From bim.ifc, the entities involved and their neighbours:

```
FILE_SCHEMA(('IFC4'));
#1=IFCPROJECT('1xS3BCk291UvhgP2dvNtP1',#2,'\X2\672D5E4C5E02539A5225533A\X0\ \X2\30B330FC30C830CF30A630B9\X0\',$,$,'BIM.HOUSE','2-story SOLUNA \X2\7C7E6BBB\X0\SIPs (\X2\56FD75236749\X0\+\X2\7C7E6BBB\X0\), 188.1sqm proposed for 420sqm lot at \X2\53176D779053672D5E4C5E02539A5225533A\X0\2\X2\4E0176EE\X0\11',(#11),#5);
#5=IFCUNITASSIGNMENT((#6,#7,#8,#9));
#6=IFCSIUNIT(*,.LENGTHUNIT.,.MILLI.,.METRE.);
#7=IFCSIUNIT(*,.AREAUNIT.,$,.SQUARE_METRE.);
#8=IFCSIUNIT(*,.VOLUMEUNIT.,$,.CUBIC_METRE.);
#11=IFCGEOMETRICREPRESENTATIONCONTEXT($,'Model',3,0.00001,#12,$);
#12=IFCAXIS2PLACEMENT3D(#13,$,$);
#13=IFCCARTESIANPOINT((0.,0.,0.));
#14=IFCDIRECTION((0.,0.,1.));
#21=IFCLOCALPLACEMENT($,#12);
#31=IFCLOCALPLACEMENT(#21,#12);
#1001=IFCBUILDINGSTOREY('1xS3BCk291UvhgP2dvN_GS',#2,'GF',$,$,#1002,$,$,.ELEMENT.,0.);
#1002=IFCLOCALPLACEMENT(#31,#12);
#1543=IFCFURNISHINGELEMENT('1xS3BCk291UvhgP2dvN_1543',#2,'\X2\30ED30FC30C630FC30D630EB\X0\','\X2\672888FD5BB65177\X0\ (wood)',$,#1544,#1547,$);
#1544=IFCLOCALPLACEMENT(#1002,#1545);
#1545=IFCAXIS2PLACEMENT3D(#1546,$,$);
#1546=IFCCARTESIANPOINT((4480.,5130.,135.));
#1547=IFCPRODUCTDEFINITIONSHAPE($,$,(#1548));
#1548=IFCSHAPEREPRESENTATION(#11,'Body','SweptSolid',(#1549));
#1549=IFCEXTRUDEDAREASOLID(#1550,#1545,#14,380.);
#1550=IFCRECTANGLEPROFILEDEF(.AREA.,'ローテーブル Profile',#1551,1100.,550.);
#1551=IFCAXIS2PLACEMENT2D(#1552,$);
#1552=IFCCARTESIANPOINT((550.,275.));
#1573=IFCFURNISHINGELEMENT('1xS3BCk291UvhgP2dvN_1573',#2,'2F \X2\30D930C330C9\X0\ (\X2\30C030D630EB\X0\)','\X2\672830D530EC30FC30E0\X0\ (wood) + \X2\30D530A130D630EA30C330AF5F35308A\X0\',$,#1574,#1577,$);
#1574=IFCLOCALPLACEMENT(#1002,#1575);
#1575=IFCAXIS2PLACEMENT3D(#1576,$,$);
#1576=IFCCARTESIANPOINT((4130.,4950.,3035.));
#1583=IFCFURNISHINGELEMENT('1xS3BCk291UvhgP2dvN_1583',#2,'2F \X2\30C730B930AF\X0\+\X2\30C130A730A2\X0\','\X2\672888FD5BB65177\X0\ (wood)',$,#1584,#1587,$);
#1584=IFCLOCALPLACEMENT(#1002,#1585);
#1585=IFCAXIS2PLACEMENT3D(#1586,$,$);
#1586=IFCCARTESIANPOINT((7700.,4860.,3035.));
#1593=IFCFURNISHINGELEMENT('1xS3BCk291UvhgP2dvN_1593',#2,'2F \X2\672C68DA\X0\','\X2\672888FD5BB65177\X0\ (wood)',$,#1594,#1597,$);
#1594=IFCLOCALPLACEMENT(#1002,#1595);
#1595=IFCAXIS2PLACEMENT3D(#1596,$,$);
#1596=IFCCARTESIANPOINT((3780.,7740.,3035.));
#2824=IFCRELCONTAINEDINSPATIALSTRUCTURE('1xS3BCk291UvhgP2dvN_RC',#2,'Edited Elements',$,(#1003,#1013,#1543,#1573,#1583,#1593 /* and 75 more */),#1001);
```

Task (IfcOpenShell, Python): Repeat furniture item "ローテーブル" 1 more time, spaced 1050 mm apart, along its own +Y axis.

```python
import ifcopenshell
import ifcopenshell.api.geometry
import ifcopenshell.api.root
import ifcopenshell.util.element
import ifcopenshell.util.placement
import ifcopenshell.util.unit

model = ifcopenshell.open("bim.ifc")
unit_scale = ifcopenshell.util.unit.calculate_unit_scale(model)


def reuse_history(source, copy):
    """copy_class also copies each property set's owner history, people and application; keep the originals."""
    for rel in copy.IsDefinedBy:
        if rel.is_a("IfcRelDefinesByProperties") and (history := rel.RelatingPropertyDefinition.OwnerHistory):
            rel.RelatingPropertyDefinition.OwnerHistory = source.OwnerHistory
            ifcopenshell.util.element.remove_deep2(model, history)


source = model.by_guid("1xS3BCk291UvhgP2dvN_1543")
base = ifcopenshell.util.placement.get_local_placement(source.ObjectPlacement)
step = base[:3, 1] * 1.05 / unit_scale

for i in range(1, 2):
    copy = ifcopenshell.api.root.copy_class(model, product=source)
    copy.Representation = ifcopenshell.util.element.copy_deep(
        model, source.Representation, exclude=["IfcGeometricRepresentationContext", "IfcRepresentationMap"]
    )
    reuse_history(source, copy)
    matrix = base.copy()
    matrix[:3, 3] += i * step
    print("added at", matrix[:3, 3].round(3) + 0.0)
    ifcopenshell.api.geometry.edit_object_placement(model, product=copy, matrix=matrix, is_si=False)

model.write("bim-out.ifc")
```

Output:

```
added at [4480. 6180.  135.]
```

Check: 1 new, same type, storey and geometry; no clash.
